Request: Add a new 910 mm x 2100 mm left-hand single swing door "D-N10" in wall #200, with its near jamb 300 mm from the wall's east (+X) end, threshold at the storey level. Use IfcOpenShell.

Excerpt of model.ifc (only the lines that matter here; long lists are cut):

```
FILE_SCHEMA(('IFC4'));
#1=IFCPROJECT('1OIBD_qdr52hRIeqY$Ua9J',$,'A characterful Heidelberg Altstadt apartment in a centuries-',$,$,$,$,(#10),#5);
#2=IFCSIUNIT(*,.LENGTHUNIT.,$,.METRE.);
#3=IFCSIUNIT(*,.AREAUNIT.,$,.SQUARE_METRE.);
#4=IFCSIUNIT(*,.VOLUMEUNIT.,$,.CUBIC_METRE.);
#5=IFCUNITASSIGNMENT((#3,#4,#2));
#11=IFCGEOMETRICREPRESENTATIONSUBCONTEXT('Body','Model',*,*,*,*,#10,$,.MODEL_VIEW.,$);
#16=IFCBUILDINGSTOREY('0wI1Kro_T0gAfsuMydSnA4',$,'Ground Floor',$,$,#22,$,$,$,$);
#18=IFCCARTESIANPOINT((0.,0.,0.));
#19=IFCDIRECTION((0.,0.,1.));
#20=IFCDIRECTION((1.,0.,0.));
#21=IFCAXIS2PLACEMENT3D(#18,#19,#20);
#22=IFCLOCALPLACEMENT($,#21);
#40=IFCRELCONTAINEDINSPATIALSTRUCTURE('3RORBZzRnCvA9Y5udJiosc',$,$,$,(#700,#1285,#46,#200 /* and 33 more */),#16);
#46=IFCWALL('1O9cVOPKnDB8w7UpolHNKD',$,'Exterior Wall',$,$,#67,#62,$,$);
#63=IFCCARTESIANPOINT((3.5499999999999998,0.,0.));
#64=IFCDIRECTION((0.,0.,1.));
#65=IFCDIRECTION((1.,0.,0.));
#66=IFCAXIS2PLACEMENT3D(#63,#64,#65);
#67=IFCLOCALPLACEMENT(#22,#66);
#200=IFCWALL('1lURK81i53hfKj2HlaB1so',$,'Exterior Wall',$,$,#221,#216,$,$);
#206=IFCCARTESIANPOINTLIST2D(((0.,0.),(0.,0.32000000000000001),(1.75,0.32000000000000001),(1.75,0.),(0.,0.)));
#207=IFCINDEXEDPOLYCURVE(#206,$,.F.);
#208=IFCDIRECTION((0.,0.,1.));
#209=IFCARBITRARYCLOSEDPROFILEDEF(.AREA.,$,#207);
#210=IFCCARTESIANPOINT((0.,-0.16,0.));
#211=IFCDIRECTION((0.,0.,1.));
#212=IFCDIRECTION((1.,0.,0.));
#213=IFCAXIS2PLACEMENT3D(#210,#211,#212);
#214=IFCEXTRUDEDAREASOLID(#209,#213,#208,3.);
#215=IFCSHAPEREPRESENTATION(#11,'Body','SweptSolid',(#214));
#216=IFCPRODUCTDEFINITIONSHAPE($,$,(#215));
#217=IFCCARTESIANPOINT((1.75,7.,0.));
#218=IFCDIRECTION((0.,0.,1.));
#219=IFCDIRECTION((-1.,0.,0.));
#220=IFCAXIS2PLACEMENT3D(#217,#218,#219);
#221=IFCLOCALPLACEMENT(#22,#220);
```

```python
import numpy as np
import ifcopenshell
import ifcopenshell.api.feature
import ifcopenshell.api.geometry
import ifcopenshell.api.root
import ifcopenshell.api.spatial
import ifcopenshell.geom
import ifcopenshell.util.element
import ifcopenshell.util.placement
import ifcopenshell.util.representation
import ifcopenshell.util.shape
import ifcopenshell.util.unit

model = ifcopenshell.open("model.ifc")
unit_scale = ifcopenshell.util.unit.calculate_unit_scale(model)
settings = ifcopenshell.geom.settings()


def volume(element):
    """Net volume in cubic metres, openings subtracted."""
    shape = ifcopenshell.geom.create_shape(settings, element)
    return ifcopenshell.util.shape.get_volume(shape.geometry)


wall = model.by_guid("1lURK81i53hfKj2HlaB1so")
storey = ifcopenshell.util.element.get_container(wall, ifc_class="IfcBuildingStorey")
context = ifcopenshell.util.representation.get_context(model, "Model", "Body", "MODEL_VIEW")
before = volume(wall)

width, height, from_end, sill = 0.91, 2.1, 0.3, 0.0  # metres

# The wall runs along its own X axis, and the end named is its -X end.
wall_shape = ifcopenshell.geom.create_shape(settings, wall)
x, y, z = ifcopenshell.util.shape.get_vertices(wall_shape.geometry).T
start = x.min() + from_end
face, thickness = float(y.min()), float(y.max() - y.min())
wall_matrix = ifcopenshell.util.placement.get_local_placement(wall.ObjectPlacement)
level = ifcopenshell.util.placement.get_local_placement(storey.ObjectPlacement)[2, 3]


def in_wall(x, y):
    """Placement at x, y metres in the wall's axes, at sill height."""
    matrix = wall_matrix.copy()
    matrix[:, 3] = wall_matrix @ np.array([x / unit_scale, y / unit_scale, 0.0, 1.0])
    matrix[2, 3] = level + sill / unit_scale
    return matrix


# Opening: a box that overshoots both wall faces by 50 mm.
opening = ifcopenshell.api.root.create_entity(model, ifc_class="IfcOpeningElement", predefined_type="OPENING")
box = ifcopenshell.api.geometry.add_wall_representation(
    model, context=context, length=width, height=height, thickness=thickness + 0.1
)
ifcopenshell.api.geometry.assign_representation(model, product=opening, representation=box)
ifcopenshell.api.geometry.edit_object_placement(model, product=opening, matrix=in_wall(start, face - 0.05), is_si=False)
ifcopenshell.api.feature.add_feature(model, feature=opening, element=wall)

door = ifcopenshell.api.root.create_entity(model, ifc_class="IfcDoor", name="D-N10", predefined_type="DOOR")
door.OverallWidth, door.OverallHeight = width / unit_scale, height / unit_scale
door.OperationType = "SINGLE_SWING_LEFT"
body = ifcopenshell.api.geometry.add_door_representation(
    model,
    context=context,
    overall_width=door.OverallWidth,
    overall_height=door.OverallHeight,
    operation_type="SINGLE_SWING_LEFT",
    lining_properties={"LiningDepth": thickness / unit_scale, "ThresholdDepth": thickness / unit_scale},
)
ifcopenshell.api.geometry.assign_representation(model, product=door, representation=body)
ifcopenshell.api.spatial.assign_container(model, products=[door], relating_structure=storey)
ifcopenshell.api.feature.add_filling(model, opening=opening, element=door)

# The lining spans the wall, so the door starts at the wall face.
ifcopenshell.api.geometry.edit_object_placement(model, product=door, matrix=in_wall(start, face), is_si=False)

after = volume(wall)

print(f"wall volume {before:.3f} -> {after:.3f} m3")

model.write("model-out.ifc")
```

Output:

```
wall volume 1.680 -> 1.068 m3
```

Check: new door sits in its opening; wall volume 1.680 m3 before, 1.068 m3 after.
